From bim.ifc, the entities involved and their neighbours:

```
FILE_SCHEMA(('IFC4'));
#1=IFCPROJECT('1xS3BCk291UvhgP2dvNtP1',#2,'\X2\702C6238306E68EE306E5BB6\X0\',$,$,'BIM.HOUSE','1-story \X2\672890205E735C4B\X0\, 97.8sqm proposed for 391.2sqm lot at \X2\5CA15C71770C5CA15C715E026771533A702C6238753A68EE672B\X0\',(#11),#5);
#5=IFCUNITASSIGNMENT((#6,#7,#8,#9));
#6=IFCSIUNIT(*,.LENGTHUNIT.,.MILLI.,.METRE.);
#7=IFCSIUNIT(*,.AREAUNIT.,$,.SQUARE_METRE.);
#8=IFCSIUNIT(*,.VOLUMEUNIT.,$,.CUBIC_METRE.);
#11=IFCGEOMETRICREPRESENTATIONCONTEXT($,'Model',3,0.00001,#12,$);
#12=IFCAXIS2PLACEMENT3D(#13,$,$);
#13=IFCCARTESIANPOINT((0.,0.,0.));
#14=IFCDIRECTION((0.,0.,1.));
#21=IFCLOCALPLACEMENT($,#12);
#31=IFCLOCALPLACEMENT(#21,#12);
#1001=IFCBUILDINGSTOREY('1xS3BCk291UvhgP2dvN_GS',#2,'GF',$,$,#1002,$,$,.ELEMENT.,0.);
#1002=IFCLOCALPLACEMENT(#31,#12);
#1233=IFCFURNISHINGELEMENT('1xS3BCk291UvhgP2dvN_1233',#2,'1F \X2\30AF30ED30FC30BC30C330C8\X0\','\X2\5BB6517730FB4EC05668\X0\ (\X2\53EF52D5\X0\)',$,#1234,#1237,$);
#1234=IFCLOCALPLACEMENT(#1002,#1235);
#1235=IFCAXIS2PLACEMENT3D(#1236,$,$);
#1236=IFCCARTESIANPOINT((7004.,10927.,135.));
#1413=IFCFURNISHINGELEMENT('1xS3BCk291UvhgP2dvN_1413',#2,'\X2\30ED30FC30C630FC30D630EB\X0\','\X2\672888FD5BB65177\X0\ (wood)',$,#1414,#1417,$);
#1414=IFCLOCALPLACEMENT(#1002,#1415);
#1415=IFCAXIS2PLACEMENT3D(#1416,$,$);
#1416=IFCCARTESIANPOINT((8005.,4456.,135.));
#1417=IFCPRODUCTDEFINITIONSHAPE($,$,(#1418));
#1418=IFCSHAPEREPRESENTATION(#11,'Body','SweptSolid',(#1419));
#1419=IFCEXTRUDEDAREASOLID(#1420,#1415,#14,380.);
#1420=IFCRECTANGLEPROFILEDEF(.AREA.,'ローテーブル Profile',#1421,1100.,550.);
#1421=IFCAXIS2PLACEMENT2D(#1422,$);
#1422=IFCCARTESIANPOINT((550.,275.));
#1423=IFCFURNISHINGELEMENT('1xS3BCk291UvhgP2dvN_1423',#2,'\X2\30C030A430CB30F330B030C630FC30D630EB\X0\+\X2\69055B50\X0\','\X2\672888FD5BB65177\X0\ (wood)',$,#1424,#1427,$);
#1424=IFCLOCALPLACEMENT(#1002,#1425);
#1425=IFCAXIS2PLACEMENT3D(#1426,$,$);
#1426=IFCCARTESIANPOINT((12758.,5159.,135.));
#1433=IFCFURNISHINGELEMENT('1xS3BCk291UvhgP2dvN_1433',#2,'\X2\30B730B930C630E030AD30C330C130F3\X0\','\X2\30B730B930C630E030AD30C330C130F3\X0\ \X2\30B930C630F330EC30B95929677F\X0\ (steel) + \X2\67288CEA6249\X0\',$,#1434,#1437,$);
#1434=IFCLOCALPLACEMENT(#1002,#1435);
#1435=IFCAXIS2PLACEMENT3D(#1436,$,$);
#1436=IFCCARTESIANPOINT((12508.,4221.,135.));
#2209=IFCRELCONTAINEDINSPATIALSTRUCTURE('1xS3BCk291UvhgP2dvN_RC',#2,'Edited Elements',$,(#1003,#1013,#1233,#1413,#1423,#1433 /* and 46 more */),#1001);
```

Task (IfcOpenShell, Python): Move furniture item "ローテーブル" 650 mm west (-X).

```python
import ifcopenshell
import ifcopenshell.api.geometry
import ifcopenshell.util.placement
import ifcopenshell.util.unit

model = ifcopenshell.open("bim.ifc")
unit_scale = ifcopenshell.util.unit.calculate_unit_scale(model)

item = model.by_id(1413)
matrix = ifcopenshell.util.placement.get_local_placement(item.ObjectPlacement)
matrix[0, 3] -= 0.65 / unit_scale
ifcopenshell.api.geometry.edit_object_placement(model, product=item, matrix=matrix, is_si=False)

print(ifcopenshell.util.placement.get_local_placement(item.ObjectPlacement).round(3) + 0.0)

model.write("bim-out.ifc")
```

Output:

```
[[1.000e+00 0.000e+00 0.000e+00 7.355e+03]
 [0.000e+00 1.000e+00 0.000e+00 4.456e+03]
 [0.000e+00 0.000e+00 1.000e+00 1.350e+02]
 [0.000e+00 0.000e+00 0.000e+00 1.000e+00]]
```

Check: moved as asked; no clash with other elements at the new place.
